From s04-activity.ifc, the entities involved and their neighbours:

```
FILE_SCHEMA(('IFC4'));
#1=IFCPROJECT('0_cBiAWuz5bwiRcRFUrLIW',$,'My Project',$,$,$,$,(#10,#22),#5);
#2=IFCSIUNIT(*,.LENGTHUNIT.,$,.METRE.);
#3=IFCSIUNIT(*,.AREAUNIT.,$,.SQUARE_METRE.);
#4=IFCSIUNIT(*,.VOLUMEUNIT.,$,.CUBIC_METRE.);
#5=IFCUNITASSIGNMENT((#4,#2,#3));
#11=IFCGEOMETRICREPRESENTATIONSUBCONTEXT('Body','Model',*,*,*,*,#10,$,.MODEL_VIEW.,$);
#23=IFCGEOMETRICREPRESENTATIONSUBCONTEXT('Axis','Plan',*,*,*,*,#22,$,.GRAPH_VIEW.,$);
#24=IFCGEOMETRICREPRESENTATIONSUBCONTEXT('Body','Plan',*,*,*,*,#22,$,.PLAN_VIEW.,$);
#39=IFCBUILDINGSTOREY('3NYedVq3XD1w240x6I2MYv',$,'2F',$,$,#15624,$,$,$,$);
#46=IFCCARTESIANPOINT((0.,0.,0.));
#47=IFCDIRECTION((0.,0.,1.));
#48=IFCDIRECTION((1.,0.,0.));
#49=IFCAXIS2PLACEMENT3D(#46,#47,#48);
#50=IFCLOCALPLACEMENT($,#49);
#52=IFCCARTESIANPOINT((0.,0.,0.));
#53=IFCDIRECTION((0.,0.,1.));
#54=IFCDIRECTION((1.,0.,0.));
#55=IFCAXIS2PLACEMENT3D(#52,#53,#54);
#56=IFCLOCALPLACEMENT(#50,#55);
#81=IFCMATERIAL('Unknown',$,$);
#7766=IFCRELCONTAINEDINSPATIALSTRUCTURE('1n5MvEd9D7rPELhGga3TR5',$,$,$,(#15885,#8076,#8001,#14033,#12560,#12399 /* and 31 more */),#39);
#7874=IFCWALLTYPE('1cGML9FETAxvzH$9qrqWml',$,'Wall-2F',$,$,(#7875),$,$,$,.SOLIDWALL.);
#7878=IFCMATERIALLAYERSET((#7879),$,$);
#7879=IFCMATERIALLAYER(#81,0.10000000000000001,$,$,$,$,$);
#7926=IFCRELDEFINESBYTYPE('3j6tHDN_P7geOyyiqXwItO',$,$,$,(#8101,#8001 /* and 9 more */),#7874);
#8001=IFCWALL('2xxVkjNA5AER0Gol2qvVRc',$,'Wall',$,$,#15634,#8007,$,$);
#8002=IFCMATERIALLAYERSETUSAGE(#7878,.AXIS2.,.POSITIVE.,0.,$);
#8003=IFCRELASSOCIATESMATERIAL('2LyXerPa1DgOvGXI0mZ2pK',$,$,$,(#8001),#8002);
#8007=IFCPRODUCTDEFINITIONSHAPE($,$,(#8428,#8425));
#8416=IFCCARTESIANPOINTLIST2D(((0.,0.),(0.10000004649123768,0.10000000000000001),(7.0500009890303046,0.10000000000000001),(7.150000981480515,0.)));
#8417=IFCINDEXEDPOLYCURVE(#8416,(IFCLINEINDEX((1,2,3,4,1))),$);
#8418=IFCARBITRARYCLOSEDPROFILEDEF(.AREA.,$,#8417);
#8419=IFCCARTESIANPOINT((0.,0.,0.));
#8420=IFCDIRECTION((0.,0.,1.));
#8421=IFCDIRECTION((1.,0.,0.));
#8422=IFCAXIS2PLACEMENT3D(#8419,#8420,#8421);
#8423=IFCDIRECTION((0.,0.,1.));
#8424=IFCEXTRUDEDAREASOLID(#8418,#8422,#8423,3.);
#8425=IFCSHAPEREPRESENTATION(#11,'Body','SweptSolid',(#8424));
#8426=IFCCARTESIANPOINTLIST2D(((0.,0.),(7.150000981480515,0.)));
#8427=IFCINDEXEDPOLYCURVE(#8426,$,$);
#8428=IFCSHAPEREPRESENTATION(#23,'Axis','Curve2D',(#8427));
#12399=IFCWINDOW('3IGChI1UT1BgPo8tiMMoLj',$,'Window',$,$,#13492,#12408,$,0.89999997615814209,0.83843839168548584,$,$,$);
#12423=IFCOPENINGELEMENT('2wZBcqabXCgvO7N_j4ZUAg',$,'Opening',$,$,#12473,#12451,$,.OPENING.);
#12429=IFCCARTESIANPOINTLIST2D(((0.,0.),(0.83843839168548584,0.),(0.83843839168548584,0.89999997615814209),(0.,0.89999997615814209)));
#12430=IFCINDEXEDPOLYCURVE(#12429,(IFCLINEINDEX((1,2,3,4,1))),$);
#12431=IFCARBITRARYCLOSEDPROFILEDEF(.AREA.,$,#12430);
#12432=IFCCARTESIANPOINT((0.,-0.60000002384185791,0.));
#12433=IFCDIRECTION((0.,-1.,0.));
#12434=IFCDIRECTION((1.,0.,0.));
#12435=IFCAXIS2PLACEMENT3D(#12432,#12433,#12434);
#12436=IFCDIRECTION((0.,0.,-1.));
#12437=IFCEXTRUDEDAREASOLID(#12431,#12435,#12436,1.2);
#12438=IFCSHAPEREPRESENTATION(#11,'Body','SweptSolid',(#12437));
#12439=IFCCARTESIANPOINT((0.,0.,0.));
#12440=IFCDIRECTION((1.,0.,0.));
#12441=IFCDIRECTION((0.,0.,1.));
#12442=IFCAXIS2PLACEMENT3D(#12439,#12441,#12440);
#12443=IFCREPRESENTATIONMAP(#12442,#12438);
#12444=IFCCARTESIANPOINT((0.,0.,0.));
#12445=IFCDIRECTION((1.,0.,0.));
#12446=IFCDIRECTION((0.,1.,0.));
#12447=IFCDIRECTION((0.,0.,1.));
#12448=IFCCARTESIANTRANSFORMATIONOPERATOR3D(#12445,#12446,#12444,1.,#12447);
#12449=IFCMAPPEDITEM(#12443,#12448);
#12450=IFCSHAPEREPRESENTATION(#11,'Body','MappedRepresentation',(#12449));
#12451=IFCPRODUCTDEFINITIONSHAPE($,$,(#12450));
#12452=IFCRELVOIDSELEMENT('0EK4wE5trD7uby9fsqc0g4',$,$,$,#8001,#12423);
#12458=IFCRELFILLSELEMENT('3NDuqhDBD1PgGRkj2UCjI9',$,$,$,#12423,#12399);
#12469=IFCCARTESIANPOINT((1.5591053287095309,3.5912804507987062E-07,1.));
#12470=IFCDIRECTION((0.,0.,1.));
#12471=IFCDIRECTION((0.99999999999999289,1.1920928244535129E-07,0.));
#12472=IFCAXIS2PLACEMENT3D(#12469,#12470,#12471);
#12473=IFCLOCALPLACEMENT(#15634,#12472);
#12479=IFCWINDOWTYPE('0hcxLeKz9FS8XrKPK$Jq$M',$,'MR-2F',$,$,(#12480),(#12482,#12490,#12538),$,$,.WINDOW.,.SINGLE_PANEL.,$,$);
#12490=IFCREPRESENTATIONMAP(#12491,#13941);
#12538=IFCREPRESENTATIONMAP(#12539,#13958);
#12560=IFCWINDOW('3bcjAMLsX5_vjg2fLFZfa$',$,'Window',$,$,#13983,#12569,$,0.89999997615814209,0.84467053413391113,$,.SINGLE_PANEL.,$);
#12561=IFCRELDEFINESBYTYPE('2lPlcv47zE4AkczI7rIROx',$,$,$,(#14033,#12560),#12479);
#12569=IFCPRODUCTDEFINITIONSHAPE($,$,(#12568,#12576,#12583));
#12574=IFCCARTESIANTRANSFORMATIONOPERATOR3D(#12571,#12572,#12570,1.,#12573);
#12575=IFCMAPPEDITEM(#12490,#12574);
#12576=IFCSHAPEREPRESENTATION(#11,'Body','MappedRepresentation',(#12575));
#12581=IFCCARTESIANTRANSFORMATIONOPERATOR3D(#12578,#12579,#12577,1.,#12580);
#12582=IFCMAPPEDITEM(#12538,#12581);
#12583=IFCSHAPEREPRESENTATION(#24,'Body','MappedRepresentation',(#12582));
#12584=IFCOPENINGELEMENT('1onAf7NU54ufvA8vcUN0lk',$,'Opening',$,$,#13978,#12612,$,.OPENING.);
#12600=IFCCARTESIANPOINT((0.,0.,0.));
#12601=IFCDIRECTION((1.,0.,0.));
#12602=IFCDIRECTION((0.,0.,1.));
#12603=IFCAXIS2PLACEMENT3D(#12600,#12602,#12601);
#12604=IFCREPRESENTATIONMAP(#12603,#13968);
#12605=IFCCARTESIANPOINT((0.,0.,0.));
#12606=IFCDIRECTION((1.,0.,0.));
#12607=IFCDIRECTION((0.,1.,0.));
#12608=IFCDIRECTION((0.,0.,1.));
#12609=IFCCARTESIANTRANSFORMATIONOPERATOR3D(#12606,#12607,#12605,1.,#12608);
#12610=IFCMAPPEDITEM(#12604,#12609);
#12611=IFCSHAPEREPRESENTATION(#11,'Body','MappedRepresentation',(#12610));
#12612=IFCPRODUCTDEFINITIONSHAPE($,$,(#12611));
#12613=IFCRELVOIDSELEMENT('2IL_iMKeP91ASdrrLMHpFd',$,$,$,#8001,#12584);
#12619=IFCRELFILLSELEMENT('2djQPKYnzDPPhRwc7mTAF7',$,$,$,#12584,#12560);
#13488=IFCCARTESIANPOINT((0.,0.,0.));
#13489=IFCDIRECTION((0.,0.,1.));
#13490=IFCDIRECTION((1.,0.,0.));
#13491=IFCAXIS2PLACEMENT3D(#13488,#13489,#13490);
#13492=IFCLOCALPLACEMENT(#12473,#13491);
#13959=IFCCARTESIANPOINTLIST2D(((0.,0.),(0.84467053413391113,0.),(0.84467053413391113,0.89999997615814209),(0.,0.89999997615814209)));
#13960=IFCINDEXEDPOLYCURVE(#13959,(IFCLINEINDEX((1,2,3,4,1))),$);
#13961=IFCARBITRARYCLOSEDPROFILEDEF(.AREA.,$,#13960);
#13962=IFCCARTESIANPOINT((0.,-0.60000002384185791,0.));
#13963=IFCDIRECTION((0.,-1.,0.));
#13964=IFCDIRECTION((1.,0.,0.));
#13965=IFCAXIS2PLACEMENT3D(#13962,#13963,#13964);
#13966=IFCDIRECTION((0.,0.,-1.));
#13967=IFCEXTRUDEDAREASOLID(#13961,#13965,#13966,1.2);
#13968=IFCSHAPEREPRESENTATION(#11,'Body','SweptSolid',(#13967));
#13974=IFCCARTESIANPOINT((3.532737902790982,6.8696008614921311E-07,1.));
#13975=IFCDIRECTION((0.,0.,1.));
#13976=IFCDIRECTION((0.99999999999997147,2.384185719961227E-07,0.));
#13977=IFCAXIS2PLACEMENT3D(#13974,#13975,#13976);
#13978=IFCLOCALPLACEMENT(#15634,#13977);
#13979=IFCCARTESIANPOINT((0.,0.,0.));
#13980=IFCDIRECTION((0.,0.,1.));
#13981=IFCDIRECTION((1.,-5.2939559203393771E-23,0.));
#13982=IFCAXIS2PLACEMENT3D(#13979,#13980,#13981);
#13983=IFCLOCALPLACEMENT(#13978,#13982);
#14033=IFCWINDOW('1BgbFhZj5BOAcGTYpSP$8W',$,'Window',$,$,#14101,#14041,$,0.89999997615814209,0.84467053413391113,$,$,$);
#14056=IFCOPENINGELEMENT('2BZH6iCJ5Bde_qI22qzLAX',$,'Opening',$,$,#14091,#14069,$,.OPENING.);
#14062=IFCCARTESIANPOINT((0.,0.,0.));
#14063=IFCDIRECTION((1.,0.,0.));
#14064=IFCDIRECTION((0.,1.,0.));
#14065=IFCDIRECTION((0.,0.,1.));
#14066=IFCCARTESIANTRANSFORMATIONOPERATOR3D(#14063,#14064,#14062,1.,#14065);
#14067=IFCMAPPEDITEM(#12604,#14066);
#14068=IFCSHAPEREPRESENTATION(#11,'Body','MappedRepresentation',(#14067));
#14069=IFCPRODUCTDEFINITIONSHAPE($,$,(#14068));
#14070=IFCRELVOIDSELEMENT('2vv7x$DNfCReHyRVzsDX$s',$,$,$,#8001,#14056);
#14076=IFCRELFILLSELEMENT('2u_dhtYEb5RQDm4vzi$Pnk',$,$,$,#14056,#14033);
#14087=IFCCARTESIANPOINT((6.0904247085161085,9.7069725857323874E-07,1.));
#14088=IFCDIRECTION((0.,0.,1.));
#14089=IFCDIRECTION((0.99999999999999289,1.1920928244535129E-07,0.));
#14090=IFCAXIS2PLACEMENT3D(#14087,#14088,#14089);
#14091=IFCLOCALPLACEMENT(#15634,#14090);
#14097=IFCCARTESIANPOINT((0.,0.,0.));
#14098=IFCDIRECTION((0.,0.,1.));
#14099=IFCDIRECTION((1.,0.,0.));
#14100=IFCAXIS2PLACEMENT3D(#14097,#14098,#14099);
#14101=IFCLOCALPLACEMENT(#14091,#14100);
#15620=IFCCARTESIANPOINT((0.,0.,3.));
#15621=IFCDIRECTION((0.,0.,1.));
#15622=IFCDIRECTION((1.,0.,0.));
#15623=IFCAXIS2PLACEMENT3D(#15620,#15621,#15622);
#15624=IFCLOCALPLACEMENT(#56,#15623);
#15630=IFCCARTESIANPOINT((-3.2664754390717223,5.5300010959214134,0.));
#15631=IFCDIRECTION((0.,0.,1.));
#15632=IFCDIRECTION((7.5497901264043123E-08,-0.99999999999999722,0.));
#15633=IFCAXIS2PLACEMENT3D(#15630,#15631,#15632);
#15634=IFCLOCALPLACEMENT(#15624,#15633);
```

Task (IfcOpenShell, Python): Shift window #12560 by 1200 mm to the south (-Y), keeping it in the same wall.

```python
import ifcopenshell
import ifcopenshell.api.geometry
import ifcopenshell.util.placement
import ifcopenshell.util.unit

model = ifcopenshell.open("s04-activity.ifc")
unit_scale = ifcopenshell.util.unit.calculate_unit_scale(model)

window = model.by_guid("3bcjAMLsX5_vjg2fLFZfa$")
opening = window.FillsVoids[0].RelatingOpeningElement
wall = opening.VoidsElements[0].RelatingBuildingElement

wall_matrix = ifcopenshell.util.placement.get_local_placement(wall.ObjectPlacement)
shift = wall_matrix[:3, 0] * 1.2 / unit_scale
before = ifcopenshell.util.placement.get_local_placement(window.ObjectPlacement)[:3, 3].copy()

# The window is placed relative to its opening, so it follows when the opening moves.
matrix = ifcopenshell.util.placement.get_local_placement(opening.ObjectPlacement)
matrix[:3, 3] += shift
ifcopenshell.api.geometry.edit_object_placement(
    model, product=opening, matrix=matrix, is_si=False, should_transform_children=True
)

after = ifcopenshell.util.placement.get_local_placement(window.ObjectPlacement)[:3, 3]
print("window moved by", (after - before).round(3) + 0.0)

model.write("s04-activity_updated.ifc")
```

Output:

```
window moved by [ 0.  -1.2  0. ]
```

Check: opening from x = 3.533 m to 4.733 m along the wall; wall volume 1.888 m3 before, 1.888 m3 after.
